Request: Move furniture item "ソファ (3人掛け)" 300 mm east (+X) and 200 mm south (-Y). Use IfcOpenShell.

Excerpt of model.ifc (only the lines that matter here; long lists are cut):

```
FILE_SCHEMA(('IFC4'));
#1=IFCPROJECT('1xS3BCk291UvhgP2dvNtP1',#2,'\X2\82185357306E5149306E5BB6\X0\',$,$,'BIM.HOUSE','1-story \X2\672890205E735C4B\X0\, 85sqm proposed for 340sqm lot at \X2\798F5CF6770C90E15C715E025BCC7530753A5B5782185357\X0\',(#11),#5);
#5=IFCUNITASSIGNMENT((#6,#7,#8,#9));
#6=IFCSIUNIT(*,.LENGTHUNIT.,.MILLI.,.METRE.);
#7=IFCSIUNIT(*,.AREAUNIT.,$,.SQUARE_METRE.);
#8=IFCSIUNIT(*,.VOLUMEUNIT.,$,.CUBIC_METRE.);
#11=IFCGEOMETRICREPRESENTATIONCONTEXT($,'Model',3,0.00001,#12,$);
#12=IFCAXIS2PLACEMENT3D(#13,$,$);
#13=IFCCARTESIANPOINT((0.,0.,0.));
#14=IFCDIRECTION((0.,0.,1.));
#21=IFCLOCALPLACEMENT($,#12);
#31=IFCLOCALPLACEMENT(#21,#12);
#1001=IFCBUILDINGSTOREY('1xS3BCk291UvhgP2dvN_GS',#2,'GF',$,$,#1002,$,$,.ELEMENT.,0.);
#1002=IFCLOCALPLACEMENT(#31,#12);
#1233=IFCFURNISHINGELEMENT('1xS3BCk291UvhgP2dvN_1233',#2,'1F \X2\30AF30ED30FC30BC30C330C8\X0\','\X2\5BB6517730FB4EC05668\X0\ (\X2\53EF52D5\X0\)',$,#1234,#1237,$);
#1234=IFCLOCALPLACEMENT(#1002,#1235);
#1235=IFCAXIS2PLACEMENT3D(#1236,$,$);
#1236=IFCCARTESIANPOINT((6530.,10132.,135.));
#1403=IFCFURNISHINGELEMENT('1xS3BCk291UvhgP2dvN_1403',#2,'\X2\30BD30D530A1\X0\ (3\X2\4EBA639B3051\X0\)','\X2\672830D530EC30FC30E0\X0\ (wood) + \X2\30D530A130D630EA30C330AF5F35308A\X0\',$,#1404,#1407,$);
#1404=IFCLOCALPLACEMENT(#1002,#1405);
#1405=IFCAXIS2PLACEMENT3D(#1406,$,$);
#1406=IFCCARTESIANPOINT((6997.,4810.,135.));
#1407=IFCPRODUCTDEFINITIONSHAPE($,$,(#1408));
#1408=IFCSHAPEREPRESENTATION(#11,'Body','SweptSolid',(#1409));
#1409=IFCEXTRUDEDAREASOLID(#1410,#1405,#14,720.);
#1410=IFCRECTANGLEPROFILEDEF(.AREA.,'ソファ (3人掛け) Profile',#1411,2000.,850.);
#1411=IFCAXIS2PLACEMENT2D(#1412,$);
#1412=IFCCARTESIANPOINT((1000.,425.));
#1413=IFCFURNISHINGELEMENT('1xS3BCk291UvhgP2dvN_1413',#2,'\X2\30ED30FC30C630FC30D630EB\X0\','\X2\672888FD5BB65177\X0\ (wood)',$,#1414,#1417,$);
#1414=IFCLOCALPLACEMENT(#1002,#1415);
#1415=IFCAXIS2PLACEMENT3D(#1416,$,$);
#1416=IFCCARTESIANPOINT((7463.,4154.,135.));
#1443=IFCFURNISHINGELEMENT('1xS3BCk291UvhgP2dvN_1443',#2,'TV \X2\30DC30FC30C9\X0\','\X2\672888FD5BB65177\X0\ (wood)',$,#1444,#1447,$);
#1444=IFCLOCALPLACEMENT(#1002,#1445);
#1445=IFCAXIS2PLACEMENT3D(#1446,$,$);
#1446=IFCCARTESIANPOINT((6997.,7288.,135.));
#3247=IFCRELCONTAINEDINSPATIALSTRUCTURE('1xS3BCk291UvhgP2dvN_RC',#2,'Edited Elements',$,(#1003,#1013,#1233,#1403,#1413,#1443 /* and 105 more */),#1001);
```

```python
import ifcopenshell
import ifcopenshell.api.geometry
import ifcopenshell.util.placement
import ifcopenshell.util.unit

model = ifcopenshell.open("model.ifc")
unit_scale = ifcopenshell.util.unit.calculate_unit_scale(model)

item = model.by_guid("1xS3BCk291UvhgP2dvN_1403")
matrix = ifcopenshell.util.placement.get_local_placement(item.ObjectPlacement)
matrix[0, 3] += 0.3 / unit_scale
matrix[1, 3] -= 0.2 / unit_scale
ifcopenshell.api.geometry.edit_object_placement(model, product=item, matrix=matrix, is_si=False)

print(ifcopenshell.util.placement.get_local_placement(item.ObjectPlacement).round(3) + 0.0)

model.write("model_edited.ifc")
```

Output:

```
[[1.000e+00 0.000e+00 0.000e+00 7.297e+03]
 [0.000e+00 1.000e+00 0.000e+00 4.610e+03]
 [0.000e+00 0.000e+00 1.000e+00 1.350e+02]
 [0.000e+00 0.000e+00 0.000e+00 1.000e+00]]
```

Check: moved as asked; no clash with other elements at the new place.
